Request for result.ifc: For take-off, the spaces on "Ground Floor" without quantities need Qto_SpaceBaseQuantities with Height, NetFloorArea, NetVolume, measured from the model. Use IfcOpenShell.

First a look at what the model holds.

```python
import ifcopenshell
import ifcopenshell.util.element
import ifcopenshell.util.unit

model = ifcopenshell.open("result.ifc")
print(model.schema)
for unit_type in ("LENGTHUNIT", "AREAUNIT", "VOLUMEUNIT"):
    print(unit_type, ifcopenshell.util.unit.calculate_unit_scale(model, unit_type))
storey = next(s for s in model.by_type("IfcBuildingStorey") if s.Name == "Ground Floor")
spaces = [e for e in ifcopenshell.util.element.get_decomposition(storey) if e.is_a("IfcSpace")]
for e in sorted(spaces, key=lambda e: e.id()):
    print(e.id(), e.is_a(), e.Name, list(ifcopenshell.util.element.get_psets(e, qtos_only=True)), sep=" | ")
```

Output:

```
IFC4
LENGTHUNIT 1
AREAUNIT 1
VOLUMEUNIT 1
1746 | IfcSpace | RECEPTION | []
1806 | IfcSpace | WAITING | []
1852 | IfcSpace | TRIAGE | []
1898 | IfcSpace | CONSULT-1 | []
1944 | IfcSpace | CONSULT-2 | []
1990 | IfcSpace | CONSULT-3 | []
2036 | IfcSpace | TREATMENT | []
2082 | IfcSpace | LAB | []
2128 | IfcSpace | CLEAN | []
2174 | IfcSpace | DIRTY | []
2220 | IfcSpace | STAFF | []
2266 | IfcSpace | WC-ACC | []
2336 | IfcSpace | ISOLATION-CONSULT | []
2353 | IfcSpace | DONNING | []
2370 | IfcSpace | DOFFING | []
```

```python
import ifcopenshell
import ifcopenshell.api.pset
import ifcopenshell.geom
import ifcopenshell.util.element
import ifcopenshell.util.shape
import ifcopenshell.util.unit

model = ifcopenshell.open("result.ifc")
unit_scale = ifcopenshell.util.unit.calculate_unit_scale(model)
area_scale = ifcopenshell.util.unit.calculate_unit_scale(model, "AREAUNIT")
volume_scale = ifcopenshell.util.unit.calculate_unit_scale(model, "VOLUMEUNIT")
settings = ifcopenshell.geom.settings()

storey = next(s for s in model.by_type("IfcBuildingStorey") if s.Name == "Ground Floor")
spaces = [e for e in ifcopenshell.util.element.get_decomposition(storey) if e.is_a("IfcSpace")]

for e in sorted(spaces, key=lambda e: e.id()):
    if ifcopenshell.util.element.get_psets(e, qtos_only=True, should_inherit=False):
        continue
    # Geometry comes back in metres, in the element's own axes.
    shape = ifcopenshell.geom.create_shape(settings, e)
    values = {
        "Height": ifcopenshell.util.shape.get_z(shape.geometry) / unit_scale,
        "NetFloorArea": ifcopenshell.util.shape.get_footprint_area(shape.geometry) / area_scale,
        "NetVolume": ifcopenshell.util.shape.get_volume(shape.geometry) / volume_scale,
    }
    qto = ifcopenshell.api.pset.add_qto(model, product=e, name="Qto_SpaceBaseQuantities")
    ifcopenshell.api.pset.edit_qto(model, qto=qto, properties=values)
    print(e.id(), {k: round(v, 3) for k, v in values.items()})

model.write("result_rev.ifc")
```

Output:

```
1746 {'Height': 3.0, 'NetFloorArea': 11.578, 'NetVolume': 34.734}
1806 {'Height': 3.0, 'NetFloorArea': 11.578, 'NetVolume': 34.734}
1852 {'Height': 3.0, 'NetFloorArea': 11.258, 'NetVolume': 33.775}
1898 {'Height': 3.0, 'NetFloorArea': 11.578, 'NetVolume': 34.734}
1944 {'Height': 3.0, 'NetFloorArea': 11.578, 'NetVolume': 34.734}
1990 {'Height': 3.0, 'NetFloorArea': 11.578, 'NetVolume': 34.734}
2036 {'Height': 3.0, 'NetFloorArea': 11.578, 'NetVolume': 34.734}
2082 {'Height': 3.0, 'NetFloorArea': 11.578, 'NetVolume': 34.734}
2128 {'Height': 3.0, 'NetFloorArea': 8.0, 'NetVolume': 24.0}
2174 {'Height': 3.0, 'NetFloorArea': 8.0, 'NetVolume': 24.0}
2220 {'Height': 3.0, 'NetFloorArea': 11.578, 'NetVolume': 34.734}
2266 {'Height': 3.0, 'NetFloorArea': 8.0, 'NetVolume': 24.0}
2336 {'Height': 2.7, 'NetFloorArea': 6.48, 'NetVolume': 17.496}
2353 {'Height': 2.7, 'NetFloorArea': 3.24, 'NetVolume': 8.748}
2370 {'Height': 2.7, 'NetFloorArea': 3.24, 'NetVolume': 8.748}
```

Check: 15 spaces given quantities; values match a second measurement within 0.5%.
